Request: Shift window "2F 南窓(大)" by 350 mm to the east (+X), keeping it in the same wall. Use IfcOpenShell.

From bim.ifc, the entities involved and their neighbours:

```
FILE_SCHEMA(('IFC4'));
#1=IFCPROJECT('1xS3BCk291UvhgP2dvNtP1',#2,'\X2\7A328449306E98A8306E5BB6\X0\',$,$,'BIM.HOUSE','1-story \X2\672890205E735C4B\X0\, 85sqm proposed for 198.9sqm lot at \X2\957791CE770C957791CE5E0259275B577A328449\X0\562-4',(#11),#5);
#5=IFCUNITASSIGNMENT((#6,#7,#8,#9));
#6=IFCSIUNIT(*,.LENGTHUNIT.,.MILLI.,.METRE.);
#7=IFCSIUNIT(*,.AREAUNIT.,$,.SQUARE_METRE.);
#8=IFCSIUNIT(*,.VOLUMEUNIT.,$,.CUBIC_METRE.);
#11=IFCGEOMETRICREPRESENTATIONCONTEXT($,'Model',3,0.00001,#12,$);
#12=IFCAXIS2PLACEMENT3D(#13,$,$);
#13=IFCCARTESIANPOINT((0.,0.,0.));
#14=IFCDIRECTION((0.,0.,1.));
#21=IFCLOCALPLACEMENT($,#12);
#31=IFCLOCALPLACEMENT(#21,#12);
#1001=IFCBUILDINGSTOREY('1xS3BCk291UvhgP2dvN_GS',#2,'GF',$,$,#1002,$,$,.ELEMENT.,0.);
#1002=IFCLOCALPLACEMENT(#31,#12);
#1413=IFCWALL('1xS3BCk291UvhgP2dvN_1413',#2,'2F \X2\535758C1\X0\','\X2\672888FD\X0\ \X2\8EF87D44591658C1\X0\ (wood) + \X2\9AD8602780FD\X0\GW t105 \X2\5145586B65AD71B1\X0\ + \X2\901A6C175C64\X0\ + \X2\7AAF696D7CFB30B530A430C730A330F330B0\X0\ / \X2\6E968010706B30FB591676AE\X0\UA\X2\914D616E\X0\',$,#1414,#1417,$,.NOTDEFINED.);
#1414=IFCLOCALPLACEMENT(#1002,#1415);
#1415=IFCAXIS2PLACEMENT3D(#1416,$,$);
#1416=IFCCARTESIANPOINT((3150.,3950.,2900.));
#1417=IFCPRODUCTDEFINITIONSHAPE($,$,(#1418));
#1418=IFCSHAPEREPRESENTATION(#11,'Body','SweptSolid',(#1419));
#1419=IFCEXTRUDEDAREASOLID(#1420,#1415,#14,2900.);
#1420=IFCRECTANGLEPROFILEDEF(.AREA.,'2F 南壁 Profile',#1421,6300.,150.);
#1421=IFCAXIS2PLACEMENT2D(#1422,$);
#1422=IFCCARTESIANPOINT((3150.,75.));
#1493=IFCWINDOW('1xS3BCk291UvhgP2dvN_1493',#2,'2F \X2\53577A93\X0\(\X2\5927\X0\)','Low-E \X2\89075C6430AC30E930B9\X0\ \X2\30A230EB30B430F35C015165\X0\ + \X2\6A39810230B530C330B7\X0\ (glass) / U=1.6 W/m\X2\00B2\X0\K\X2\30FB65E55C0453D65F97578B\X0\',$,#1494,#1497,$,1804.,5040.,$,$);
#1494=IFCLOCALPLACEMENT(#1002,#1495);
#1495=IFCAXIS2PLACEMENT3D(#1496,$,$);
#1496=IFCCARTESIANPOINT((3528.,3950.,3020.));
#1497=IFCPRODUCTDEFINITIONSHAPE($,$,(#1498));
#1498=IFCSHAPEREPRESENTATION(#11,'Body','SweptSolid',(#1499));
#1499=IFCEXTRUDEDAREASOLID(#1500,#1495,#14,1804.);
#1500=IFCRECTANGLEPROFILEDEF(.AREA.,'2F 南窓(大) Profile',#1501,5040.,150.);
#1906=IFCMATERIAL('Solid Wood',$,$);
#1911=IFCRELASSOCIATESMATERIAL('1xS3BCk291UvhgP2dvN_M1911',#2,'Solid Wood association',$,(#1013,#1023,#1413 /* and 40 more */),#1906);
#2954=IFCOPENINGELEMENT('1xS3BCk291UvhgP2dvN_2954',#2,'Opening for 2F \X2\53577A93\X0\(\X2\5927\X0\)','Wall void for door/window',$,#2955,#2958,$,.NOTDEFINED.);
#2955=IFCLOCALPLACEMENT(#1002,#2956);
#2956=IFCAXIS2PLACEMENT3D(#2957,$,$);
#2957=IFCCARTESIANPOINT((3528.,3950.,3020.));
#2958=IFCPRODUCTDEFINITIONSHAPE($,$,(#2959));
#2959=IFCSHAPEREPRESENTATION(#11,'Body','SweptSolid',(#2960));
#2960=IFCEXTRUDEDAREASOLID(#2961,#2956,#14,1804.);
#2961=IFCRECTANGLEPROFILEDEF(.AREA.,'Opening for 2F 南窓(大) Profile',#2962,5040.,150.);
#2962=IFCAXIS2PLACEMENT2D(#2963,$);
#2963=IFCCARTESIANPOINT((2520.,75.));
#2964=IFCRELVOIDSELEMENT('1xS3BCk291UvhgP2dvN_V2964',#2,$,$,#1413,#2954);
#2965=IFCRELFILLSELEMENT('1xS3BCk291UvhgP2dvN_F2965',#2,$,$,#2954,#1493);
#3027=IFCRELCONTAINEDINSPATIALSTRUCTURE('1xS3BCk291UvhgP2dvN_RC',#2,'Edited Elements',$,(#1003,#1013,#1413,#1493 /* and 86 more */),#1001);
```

```python
import ifcopenshell
import ifcopenshell.api.geometry
import ifcopenshell.util.placement

model = ifcopenshell.open("bim.ifc")

window = model.by_guid("1xS3BCk291UvhgP2dvN_1493")
opening = window.FillsVoids[0].RelatingOpeningElement
wall = opening.VoidsElements[0].RelatingBuildingElement

wall_matrix = ifcopenshell.util.placement.get_local_placement(wall.ObjectPlacement)
shift = wall_matrix[:3, 0] * 350.0
before = ifcopenshell.util.placement.get_local_placement(window.ObjectPlacement)[:3, 3].copy()

# The window is not placed relative to its opening, so move both.
for product in (opening, window):
    matrix = ifcopenshell.util.placement.get_local_placement(product.ObjectPlacement)
    matrix[:3, 3] += shift
    ifcopenshell.api.geometry.edit_object_placement(model, product=product, matrix=matrix, is_si=False)

after = ifcopenshell.util.placement.get_local_placement(window.ObjectPlacement)[:3, 3]
print("window moved by", (after - before).round(3) + 0.0)

model.write("bim-out.ifc")
```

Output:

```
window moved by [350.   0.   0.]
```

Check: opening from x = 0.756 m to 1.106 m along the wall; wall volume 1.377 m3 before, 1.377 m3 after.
